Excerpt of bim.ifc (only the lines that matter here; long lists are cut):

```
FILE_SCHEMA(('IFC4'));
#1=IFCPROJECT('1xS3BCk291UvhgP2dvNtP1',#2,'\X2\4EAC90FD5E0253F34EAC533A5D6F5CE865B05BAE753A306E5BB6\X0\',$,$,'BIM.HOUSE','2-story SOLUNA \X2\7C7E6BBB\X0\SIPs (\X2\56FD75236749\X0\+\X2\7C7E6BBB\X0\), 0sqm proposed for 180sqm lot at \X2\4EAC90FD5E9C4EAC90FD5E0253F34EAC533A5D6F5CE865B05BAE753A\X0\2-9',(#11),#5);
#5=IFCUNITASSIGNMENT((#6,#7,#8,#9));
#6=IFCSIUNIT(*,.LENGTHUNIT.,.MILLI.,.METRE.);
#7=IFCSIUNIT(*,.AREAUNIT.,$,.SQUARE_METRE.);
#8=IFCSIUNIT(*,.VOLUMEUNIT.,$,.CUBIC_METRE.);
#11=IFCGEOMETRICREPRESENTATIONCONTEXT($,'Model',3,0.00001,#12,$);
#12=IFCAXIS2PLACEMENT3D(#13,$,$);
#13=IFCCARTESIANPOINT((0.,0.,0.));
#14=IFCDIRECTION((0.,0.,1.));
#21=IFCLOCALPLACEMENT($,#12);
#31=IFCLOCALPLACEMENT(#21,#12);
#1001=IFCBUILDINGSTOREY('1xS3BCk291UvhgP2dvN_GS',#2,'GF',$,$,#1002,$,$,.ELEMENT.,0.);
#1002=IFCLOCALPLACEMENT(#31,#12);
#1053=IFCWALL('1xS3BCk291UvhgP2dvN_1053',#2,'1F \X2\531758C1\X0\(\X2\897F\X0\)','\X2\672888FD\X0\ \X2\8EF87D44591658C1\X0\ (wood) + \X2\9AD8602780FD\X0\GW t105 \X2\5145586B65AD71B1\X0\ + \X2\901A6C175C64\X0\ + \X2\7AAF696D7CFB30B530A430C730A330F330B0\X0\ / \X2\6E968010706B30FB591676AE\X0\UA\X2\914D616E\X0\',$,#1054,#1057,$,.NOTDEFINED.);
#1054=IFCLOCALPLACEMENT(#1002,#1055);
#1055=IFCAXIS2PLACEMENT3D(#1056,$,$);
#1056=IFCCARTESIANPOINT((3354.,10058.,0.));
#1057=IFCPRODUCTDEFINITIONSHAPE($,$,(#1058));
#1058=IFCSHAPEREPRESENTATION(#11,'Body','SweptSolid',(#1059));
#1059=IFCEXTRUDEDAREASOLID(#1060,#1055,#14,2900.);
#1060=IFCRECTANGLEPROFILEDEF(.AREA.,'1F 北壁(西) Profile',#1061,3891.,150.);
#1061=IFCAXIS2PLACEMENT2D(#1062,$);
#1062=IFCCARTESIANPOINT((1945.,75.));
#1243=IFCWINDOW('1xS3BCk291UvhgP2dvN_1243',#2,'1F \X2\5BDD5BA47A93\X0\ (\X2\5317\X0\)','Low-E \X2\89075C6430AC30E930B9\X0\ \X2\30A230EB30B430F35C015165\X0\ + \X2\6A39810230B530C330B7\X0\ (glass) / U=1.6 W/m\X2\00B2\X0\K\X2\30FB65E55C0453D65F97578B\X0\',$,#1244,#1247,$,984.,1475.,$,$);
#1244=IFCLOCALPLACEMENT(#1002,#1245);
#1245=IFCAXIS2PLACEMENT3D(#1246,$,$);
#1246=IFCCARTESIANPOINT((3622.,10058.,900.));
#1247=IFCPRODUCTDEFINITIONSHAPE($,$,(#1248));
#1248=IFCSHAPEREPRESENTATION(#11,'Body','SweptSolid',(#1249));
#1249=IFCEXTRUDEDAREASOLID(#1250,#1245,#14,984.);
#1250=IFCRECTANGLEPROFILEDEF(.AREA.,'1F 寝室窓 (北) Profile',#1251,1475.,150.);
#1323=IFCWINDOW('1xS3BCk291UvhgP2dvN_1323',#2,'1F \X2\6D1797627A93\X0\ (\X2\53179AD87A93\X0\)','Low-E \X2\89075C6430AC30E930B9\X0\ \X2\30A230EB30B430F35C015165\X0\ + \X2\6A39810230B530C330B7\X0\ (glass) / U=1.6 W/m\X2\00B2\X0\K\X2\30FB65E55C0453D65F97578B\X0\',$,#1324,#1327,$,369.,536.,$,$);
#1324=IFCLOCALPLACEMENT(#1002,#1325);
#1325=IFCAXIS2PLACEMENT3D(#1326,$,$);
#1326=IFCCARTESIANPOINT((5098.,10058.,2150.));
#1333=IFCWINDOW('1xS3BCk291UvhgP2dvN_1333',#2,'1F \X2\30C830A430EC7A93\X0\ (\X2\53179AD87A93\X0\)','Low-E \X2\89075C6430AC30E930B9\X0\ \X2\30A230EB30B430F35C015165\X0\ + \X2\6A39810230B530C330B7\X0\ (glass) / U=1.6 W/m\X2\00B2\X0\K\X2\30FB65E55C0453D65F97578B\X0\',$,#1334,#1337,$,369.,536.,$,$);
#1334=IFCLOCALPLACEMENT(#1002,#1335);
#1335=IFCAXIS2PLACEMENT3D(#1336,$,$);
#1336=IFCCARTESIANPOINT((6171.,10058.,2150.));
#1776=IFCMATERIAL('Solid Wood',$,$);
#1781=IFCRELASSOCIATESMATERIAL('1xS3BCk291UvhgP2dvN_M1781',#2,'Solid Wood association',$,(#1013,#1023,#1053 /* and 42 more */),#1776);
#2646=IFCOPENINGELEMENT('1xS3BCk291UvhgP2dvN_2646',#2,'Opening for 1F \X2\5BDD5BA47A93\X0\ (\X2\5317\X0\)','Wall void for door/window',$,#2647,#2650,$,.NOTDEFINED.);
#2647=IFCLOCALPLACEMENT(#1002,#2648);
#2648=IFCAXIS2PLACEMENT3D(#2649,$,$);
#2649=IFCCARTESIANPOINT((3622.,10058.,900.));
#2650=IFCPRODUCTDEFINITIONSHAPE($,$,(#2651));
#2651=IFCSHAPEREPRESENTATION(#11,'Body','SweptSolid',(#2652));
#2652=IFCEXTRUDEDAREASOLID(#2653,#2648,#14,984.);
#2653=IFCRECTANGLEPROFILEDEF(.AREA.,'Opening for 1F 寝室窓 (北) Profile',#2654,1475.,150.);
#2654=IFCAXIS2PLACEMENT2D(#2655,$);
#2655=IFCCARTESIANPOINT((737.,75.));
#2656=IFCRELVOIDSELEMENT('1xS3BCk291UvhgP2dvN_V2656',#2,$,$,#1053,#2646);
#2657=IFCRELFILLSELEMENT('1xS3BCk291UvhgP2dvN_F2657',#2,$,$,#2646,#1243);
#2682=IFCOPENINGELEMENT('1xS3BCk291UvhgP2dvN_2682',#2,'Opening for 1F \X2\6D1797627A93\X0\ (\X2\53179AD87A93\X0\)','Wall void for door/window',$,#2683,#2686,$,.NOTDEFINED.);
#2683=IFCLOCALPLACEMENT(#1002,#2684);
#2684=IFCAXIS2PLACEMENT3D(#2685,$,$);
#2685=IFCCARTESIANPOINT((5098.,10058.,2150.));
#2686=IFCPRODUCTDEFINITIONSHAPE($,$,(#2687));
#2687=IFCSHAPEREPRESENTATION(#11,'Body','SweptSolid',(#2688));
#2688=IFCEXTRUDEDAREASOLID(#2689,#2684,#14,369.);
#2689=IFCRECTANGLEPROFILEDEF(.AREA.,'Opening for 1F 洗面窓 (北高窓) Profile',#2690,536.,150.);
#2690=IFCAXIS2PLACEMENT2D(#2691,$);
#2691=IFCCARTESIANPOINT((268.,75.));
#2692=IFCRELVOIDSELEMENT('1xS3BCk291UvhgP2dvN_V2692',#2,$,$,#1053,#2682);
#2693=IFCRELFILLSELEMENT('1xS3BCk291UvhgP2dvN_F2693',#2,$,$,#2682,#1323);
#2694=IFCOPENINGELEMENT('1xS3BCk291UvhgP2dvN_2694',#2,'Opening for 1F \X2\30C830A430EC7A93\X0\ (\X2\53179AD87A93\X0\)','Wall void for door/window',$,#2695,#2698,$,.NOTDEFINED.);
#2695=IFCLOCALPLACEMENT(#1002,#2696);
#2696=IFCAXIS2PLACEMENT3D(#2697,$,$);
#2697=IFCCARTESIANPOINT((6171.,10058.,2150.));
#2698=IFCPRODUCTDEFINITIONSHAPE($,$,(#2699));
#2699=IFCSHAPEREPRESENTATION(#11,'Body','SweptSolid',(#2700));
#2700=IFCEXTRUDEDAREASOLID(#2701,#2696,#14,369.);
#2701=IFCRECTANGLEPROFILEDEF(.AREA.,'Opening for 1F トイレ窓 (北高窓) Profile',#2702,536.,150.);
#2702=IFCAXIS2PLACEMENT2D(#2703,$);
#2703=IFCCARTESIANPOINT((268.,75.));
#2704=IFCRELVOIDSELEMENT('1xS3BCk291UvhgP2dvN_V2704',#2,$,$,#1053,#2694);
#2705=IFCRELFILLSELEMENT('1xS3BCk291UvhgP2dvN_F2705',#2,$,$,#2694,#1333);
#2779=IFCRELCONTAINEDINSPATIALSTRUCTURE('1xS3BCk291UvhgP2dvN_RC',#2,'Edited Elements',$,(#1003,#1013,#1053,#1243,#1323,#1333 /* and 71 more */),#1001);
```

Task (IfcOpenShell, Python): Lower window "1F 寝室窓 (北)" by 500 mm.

```python
import numpy as np
import ifcopenshell
import ifcopenshell.api.geometry
import ifcopenshell.util.placement
import ifcopenshell.util.unit

model = ifcopenshell.open("bim.ifc")
unit_scale = ifcopenshell.util.unit.calculate_unit_scale(model)

window = model.by_guid("1xS3BCk291UvhgP2dvN_1243")
opening = window.FillsVoids[0].RelatingOpeningElement
dz = -0.5 / unit_scale

shift = np.array([0.0, 0.0, dz])
# The window is not placed relative to its opening, so move both.
for product in (opening, window):
    matrix = ifcopenshell.util.placement.get_local_placement(product.ObjectPlacement)
    matrix[:3, 3] += shift
    ifcopenshell.api.geometry.edit_object_placement(model, product=product, matrix=matrix, is_si=False)

print(f"moved by {dz * unit_scale:+.3f} m")

model.write("bim-out.ifc")
```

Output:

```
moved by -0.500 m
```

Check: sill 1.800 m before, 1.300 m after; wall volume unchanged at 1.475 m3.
